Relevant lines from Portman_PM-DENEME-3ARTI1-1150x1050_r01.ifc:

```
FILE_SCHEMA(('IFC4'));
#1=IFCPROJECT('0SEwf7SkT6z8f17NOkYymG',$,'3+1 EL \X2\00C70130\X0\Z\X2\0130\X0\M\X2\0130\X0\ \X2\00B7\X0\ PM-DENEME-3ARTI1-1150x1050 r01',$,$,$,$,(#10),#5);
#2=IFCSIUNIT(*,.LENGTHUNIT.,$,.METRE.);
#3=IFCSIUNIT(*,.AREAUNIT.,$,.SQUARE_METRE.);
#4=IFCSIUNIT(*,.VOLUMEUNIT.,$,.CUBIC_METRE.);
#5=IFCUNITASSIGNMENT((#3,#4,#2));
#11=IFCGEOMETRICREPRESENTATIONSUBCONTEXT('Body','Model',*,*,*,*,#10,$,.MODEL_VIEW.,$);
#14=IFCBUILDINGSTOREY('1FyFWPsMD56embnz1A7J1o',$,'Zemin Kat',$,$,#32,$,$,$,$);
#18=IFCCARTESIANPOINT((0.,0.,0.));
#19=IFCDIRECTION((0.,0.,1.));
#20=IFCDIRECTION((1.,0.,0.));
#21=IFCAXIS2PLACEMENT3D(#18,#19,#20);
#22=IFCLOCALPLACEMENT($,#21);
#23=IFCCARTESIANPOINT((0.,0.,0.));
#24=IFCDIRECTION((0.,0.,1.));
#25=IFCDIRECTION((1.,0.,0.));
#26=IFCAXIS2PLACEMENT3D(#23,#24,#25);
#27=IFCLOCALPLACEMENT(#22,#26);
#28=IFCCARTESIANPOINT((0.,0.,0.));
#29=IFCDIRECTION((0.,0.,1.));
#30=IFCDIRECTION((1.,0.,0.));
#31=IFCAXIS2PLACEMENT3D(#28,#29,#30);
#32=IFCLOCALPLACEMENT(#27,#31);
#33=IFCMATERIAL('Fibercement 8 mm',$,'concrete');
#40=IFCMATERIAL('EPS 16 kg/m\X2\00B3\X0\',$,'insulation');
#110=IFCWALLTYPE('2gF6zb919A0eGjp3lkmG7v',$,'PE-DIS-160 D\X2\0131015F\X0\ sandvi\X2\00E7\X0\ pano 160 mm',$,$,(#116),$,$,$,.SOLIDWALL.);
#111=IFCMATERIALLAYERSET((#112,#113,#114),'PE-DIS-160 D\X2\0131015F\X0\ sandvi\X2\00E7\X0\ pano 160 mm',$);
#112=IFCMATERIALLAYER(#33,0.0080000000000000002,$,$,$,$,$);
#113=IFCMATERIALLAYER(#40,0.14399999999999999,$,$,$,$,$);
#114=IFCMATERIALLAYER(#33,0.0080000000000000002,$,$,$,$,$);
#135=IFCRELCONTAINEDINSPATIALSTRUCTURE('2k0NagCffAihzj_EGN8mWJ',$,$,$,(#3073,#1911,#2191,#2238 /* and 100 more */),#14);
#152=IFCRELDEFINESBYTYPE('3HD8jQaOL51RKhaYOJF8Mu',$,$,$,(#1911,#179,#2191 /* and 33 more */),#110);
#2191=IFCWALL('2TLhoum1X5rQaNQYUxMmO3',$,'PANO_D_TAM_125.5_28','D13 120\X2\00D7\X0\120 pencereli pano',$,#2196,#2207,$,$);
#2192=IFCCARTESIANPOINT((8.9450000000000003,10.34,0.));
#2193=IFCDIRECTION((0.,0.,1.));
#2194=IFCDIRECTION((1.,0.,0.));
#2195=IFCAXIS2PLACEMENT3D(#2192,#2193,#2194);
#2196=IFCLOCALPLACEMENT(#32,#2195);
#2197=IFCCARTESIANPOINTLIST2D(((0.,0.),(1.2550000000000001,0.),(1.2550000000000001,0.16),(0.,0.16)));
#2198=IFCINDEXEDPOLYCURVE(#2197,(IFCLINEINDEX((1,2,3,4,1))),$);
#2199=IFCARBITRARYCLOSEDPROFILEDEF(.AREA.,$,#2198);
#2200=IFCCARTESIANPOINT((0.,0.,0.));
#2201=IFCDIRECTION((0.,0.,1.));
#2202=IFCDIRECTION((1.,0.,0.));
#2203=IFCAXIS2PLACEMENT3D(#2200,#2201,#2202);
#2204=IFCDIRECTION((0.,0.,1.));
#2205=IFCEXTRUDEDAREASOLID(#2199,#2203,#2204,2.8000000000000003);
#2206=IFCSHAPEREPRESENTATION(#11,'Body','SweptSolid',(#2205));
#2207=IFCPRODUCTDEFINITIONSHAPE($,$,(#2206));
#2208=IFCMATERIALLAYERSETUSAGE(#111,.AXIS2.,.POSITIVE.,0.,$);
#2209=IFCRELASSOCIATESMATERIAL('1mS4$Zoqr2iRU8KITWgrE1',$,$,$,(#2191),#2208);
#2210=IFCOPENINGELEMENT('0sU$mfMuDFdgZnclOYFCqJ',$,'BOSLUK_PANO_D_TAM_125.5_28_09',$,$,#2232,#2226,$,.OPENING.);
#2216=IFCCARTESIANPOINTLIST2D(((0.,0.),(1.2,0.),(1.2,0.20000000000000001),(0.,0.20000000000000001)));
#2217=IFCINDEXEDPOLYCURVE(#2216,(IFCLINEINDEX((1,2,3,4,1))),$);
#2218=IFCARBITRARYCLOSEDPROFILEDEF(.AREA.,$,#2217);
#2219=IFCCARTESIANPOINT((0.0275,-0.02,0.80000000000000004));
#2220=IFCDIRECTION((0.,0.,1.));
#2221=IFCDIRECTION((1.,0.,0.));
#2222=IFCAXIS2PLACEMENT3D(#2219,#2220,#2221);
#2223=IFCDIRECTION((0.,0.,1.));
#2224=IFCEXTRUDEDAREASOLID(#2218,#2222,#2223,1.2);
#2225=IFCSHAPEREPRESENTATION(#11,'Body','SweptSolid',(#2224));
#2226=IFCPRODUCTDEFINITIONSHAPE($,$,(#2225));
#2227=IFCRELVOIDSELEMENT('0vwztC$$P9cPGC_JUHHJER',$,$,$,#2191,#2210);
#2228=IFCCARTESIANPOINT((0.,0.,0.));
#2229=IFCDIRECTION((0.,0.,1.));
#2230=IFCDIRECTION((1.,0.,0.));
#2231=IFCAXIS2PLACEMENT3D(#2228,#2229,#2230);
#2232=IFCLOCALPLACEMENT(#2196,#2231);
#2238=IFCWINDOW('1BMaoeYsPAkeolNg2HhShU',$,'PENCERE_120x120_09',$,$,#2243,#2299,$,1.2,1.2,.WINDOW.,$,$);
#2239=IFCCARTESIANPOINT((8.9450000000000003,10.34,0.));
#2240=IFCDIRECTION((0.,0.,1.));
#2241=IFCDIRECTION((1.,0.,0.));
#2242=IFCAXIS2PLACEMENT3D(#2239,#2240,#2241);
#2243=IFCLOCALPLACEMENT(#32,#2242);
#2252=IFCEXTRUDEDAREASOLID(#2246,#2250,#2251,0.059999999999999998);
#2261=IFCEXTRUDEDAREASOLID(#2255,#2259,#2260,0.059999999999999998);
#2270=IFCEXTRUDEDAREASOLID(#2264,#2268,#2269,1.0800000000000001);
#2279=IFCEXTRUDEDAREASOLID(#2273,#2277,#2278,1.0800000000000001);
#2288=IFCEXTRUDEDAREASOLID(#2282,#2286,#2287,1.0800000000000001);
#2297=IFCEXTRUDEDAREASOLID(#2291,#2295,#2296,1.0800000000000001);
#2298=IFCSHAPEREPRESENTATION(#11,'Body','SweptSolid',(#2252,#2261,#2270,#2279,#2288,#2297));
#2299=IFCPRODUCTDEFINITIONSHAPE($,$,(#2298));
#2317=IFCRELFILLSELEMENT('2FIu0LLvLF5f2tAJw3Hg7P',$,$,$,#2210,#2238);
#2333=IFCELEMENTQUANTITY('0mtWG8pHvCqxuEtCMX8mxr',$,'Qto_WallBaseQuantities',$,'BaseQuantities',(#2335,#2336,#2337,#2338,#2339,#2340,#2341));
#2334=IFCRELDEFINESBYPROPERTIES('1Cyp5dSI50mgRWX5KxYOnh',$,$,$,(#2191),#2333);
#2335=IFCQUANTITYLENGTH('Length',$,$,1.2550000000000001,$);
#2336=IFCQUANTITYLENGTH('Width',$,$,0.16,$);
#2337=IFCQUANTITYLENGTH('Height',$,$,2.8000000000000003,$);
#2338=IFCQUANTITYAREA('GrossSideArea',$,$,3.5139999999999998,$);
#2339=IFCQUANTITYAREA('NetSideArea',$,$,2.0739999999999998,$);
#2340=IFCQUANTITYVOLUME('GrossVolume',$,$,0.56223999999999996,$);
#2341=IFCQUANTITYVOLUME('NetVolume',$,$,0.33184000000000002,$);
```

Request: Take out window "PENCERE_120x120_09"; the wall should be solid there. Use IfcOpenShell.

```python
import ifcopenshell
import ifcopenshell.api.feature
import ifcopenshell.api.pset
import ifcopenshell.api.root
import ifcopenshell.geom
import ifcopenshell.util.element
import ifcopenshell.util.shape
import ifcopenshell.util.unit

model = ifcopenshell.open("Portman_PM-DENEME-3ARTI1-1150x1050_r01.ifc")
area_scale = ifcopenshell.util.unit.calculate_unit_scale(model, "AREAUNIT")
volume_scale = ifcopenshell.util.unit.calculate_unit_scale(model, "VOLUMEUNIT")
settings = ifcopenshell.geom.settings()


def volume(element):
    """Net volume in cubic metres, openings subtracted."""
    shape = ifcopenshell.geom.create_shape(settings, element)
    return ifcopenshell.util.shape.get_volume(shape.geometry)


window = model.by_guid("1BMaoeYsPAkeolNg2HhShU")
opening = window.FillsVoids[0].RelatingOpeningElement
wall = opening.VoidsElements[0].RelatingBuildingElement
before = volume(wall)

ifcopenshell.api.root.remove_product(model, product=window)
ifcopenshell.api.feature.remove_feature(model, feature=opening)

after = volume(wall)
thickness = 0.16  # wall thickness in metres

# Update the wall's stored quantities.
qto = model.by_id(ifcopenshell.util.element.get_pset(wall, "Qto_WallBaseQuantities", should_inherit=False)["id"])
ifcopenshell.api.pset.edit_qto(model, qto=qto, properties={
    "NetSideArea": after / thickness / area_scale,
    "NetVolume": after / volume_scale,
})

print(f"wall volume {before:.3f} -> {after:.3f} m3")

model.write("Portman_PM-DENEME-3ARTI1-1150x1050_r01_edited.ifc")
```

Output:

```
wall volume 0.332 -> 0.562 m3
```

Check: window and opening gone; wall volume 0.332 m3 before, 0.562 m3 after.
